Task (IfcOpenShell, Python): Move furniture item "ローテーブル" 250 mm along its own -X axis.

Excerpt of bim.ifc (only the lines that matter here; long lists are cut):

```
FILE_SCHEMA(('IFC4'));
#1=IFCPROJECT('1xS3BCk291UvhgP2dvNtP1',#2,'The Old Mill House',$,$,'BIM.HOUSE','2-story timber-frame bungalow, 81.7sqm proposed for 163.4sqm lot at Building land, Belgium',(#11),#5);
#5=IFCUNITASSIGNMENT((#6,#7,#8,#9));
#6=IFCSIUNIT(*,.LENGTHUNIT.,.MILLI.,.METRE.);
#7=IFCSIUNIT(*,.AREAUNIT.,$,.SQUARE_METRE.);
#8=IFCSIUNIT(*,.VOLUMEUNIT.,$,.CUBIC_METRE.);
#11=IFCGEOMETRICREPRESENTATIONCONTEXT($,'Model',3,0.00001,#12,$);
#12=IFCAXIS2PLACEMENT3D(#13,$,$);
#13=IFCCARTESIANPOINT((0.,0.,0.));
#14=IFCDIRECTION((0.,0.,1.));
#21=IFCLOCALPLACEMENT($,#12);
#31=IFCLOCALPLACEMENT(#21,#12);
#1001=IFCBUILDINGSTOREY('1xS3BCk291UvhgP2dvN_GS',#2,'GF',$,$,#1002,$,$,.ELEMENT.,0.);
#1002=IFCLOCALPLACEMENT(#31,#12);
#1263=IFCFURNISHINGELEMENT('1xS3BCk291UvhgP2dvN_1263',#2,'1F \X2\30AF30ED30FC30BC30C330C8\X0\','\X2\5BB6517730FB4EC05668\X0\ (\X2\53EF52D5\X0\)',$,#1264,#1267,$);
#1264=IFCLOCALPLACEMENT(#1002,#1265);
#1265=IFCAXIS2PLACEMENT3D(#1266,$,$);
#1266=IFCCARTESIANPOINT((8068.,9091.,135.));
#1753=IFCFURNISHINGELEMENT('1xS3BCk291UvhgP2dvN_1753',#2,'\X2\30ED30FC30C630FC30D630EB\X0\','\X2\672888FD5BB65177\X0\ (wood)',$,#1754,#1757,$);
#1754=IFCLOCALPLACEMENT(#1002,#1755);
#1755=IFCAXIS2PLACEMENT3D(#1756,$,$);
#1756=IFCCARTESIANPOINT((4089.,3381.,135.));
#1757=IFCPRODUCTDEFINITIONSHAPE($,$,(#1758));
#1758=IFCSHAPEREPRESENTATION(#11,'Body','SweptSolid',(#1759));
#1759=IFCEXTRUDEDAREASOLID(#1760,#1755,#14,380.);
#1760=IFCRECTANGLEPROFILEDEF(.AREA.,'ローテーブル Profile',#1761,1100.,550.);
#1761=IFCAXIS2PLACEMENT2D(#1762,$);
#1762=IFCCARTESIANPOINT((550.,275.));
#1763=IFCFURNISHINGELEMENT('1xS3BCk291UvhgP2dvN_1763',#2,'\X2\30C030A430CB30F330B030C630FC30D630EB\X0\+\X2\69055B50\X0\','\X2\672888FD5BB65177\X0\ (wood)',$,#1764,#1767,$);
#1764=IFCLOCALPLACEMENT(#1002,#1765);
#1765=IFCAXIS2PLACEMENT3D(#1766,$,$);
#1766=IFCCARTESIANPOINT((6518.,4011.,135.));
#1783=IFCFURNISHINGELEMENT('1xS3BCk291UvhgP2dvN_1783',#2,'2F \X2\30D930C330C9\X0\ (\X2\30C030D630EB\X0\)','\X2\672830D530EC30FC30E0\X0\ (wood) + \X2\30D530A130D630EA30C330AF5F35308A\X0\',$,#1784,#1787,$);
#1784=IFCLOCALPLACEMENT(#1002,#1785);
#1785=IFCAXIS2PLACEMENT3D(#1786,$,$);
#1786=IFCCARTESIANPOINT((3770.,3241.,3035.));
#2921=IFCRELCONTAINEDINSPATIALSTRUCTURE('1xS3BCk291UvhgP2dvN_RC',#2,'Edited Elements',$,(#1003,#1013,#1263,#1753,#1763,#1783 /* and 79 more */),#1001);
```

```python
import ifcopenshell
import ifcopenshell.api.geometry
import ifcopenshell.util.placement
import ifcopenshell.util.unit

model = ifcopenshell.open("bim.ifc")
unit_scale = ifcopenshell.util.unit.calculate_unit_scale(model)

item = model.by_guid("1xS3BCk291UvhgP2dvN_1753")
matrix = ifcopenshell.util.placement.get_local_placement(item.ObjectPlacement)
matrix[:3, 3] -= matrix[:3, 0] * 0.25 / unit_scale
ifcopenshell.api.geometry.edit_object_placement(model, product=item, matrix=matrix, is_si=False)

print(ifcopenshell.util.placement.get_local_placement(item.ObjectPlacement).round(3) + 0.0)

model.write("bim_updated.ifc")
```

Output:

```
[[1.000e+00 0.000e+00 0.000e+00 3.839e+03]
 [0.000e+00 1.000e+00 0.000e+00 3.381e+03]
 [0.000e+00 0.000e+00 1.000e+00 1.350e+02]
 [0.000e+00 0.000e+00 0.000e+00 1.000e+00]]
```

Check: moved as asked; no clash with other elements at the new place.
